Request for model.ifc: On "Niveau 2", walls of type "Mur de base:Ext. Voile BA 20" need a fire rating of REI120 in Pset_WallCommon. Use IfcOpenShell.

First a look at what the model holds.

```python
import ifcopenshell
import ifcopenshell.util.element

model = ifcopenshell.open("model.ifc")
print(model.schema)
storey = next(s for s in model.by_type("IfcBuildingStorey") if s.Name == "Niveau 2")
walls = [e for e in ifcopenshell.util.element.get_decomposition(storey) if e.is_a("IfcWall")]
seen = {}
for e in walls:
    element_type = ifcopenshell.util.element.get_type(e)
    key = (element_type.Name if element_type != e and element_type else None, ifcopenshell.util.element.get_pset(e, "Pset_WallCommon", "FireRating"))
    seen[key] = seen.get(key, 0) + 1
for (name, value), count in sorted(seen.items(), key=str):
    print(count, "x", name, "|", value)
```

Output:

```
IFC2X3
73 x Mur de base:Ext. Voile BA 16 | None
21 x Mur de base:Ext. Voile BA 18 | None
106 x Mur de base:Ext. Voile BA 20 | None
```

```python
import ifcopenshell
import ifcopenshell.api.pset
import ifcopenshell.util.element

model = ifcopenshell.open("model.ifc")

storey = next(s for s in model.by_type("IfcBuildingStorey") if s.Name == "Niveau 2")
walls = [e for e in ifcopenshell.util.element.get_decomposition(storey) if e.is_a("IfcWall")]

count = 0
for e in walls:
    element_type = ifcopenshell.util.element.get_type(e)
    if element_type in (None, e) or element_type.Name != "Mur de base:Ext. Voile BA 20":
        continue
    # add_pset returns the element's existing set when there is one.
    pset = ifcopenshell.api.pset.add_pset(model, product=e, name="Pset_WallCommon")
    ifcopenshell.api.pset.edit_pset(model, pset=pset, properties={"FireRating": "REI120"})
    count += 1

print(count, "walls updated")

model.write("model_v2.ifc")
```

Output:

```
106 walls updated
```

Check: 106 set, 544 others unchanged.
